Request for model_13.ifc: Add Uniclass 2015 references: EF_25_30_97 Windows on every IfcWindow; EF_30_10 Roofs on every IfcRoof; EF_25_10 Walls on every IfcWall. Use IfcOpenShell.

First a look at what the model holds.

```python
import ifcopenshell

model = ifcopenshell.open("model_13.ifc")
print(model.schema)
print("classifications:", [c.Name for c in model.by_type("IfcClassification")])
for ifc_class in ("IfcDoor", "IfcRoof", "IfcStair", "IfcWall", "IfcWindow"):
    print(ifc_class, len(model.by_type(ifc_class)))
```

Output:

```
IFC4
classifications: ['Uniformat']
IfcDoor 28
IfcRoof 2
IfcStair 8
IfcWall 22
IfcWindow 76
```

```python
import ifcopenshell
import ifcopenshell.api.classification

model = ifcopenshell.open("model_13.ifc")

system = ifcopenshell.api.classification.add_classification(model, classification="Uniclass 2015")

codes = {
    "IfcWindow": ("EF_25_30_97", "Windows"),
    "IfcRoof": ("EF_30_10", "Roofs"),
    "IfcWall": ("EF_25_10", "Walls"),
}
for ifc_class, (code, name) in codes.items():
    products = model.by_type(ifc_class)
    ifcopenshell.api.classification.add_reference(
        model, products=products, classification=system, identification=code, name=name
    )
    print(code, len(products))

model.write("model_13-out.ifc")
```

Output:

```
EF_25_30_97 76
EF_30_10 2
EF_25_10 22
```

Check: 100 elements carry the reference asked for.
